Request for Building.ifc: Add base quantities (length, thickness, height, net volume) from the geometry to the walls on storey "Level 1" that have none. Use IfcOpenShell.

First a look at what the model holds.

```python
import ifcopenshell
import ifcopenshell.util.element
import ifcopenshell.util.unit

model = ifcopenshell.open("Building.ifc")
print(model.schema)
for unit_type in ("LENGTHUNIT", "AREAUNIT", "VOLUMEUNIT"):
    print(unit_type, ifcopenshell.util.unit.calculate_unit_scale(model, unit_type))
storey = next(s for s in model.by_type("IfcBuildingStorey") if s.Name == "Level 1")
walls = [e for e in ifcopenshell.util.element.get_decomposition(storey) if e.is_a("IfcWall")]
for e in sorted(walls, key=lambda e: e.id()):
    print(e.id(), e.is_a(), e.Name, list(ifcopenshell.util.element.get_psets(e, qtos_only=True)), sep=" | ")
```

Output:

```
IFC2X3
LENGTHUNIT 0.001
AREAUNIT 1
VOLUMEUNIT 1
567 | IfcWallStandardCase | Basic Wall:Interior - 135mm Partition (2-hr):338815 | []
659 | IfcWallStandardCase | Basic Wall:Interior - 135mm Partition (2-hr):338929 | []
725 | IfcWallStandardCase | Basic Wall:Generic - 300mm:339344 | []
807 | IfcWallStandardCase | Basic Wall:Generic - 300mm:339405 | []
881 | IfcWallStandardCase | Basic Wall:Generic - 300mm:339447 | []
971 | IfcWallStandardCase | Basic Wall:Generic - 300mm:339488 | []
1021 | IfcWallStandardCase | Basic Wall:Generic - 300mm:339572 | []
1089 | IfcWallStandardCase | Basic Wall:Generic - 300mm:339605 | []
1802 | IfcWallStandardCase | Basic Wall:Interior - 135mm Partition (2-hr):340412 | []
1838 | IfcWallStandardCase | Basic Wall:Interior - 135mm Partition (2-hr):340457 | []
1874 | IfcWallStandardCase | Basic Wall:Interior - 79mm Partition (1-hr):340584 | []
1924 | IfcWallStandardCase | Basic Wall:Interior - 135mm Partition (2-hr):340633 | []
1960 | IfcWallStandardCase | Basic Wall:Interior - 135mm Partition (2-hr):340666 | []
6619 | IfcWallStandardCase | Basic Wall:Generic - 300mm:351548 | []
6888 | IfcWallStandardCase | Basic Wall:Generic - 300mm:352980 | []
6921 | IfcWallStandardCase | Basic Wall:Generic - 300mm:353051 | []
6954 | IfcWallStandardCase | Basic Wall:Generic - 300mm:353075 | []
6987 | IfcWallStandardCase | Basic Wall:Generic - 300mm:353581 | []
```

```python
import ifcopenshell
import ifcopenshell.api.pset
import ifcopenshell.geom
import ifcopenshell.util.element
import ifcopenshell.util.shape
import ifcopenshell.util.unit

model = ifcopenshell.open("Building.ifc")
unit_scale = ifcopenshell.util.unit.calculate_unit_scale(model)
volume_scale = ifcopenshell.util.unit.calculate_unit_scale(model, "VOLUMEUNIT")
settings = ifcopenshell.geom.settings()

storey = next(s for s in model.by_type("IfcBuildingStorey") if s.Name == "Level 1")
walls = [e for e in ifcopenshell.util.element.get_decomposition(storey) if e.is_a("IfcWall")]

for e in sorted(walls, key=lambda e: e.id()):
    if ifcopenshell.util.element.get_psets(e, qtos_only=True, should_inherit=False):
        continue
    # Geometry comes back in metres, in the element's own axes.
    shape = ifcopenshell.geom.create_shape(settings, e)
    values = {
        "Length": ifcopenshell.util.shape.get_x(shape.geometry) / unit_scale,
        "Width": ifcopenshell.util.shape.get_y(shape.geometry) / unit_scale,
        "Height": ifcopenshell.util.shape.get_z(shape.geometry) / unit_scale,
        "NetVolume": ifcopenshell.util.shape.get_volume(shape.geometry) / volume_scale,
    }
    qto = ifcopenshell.api.pset.add_qto(model, product=e, name="BaseQuantities")
    ifcopenshell.api.pset.edit_qto(model, qto=qto, properties=values)
    print(e.id(), {k: round(v, 3) for k, v in values.items()})

model.write("Building_edited.ifc")
```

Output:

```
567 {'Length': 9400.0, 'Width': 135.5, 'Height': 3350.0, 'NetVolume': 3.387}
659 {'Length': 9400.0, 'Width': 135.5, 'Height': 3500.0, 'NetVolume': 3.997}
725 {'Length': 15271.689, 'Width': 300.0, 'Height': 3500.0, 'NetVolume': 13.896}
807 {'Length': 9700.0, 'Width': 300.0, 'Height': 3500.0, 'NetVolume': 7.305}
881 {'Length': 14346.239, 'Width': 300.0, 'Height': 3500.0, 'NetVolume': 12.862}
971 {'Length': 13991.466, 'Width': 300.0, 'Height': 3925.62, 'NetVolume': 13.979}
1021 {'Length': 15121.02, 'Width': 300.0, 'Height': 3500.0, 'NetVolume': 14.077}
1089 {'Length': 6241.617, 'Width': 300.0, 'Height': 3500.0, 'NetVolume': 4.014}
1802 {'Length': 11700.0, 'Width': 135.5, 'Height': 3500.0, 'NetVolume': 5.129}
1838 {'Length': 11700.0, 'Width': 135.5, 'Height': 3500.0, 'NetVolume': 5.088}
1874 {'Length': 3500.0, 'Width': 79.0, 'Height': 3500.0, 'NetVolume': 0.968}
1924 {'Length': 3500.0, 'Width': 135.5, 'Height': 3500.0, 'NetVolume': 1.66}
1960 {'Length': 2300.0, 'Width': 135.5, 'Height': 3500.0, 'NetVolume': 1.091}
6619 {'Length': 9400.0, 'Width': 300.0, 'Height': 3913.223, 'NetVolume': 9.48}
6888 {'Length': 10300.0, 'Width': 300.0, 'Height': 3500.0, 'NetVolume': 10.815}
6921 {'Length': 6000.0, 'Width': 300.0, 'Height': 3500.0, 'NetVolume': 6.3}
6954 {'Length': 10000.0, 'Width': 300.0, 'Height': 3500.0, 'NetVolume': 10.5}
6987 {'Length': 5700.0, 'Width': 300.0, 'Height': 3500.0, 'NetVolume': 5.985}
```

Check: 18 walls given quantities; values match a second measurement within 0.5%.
